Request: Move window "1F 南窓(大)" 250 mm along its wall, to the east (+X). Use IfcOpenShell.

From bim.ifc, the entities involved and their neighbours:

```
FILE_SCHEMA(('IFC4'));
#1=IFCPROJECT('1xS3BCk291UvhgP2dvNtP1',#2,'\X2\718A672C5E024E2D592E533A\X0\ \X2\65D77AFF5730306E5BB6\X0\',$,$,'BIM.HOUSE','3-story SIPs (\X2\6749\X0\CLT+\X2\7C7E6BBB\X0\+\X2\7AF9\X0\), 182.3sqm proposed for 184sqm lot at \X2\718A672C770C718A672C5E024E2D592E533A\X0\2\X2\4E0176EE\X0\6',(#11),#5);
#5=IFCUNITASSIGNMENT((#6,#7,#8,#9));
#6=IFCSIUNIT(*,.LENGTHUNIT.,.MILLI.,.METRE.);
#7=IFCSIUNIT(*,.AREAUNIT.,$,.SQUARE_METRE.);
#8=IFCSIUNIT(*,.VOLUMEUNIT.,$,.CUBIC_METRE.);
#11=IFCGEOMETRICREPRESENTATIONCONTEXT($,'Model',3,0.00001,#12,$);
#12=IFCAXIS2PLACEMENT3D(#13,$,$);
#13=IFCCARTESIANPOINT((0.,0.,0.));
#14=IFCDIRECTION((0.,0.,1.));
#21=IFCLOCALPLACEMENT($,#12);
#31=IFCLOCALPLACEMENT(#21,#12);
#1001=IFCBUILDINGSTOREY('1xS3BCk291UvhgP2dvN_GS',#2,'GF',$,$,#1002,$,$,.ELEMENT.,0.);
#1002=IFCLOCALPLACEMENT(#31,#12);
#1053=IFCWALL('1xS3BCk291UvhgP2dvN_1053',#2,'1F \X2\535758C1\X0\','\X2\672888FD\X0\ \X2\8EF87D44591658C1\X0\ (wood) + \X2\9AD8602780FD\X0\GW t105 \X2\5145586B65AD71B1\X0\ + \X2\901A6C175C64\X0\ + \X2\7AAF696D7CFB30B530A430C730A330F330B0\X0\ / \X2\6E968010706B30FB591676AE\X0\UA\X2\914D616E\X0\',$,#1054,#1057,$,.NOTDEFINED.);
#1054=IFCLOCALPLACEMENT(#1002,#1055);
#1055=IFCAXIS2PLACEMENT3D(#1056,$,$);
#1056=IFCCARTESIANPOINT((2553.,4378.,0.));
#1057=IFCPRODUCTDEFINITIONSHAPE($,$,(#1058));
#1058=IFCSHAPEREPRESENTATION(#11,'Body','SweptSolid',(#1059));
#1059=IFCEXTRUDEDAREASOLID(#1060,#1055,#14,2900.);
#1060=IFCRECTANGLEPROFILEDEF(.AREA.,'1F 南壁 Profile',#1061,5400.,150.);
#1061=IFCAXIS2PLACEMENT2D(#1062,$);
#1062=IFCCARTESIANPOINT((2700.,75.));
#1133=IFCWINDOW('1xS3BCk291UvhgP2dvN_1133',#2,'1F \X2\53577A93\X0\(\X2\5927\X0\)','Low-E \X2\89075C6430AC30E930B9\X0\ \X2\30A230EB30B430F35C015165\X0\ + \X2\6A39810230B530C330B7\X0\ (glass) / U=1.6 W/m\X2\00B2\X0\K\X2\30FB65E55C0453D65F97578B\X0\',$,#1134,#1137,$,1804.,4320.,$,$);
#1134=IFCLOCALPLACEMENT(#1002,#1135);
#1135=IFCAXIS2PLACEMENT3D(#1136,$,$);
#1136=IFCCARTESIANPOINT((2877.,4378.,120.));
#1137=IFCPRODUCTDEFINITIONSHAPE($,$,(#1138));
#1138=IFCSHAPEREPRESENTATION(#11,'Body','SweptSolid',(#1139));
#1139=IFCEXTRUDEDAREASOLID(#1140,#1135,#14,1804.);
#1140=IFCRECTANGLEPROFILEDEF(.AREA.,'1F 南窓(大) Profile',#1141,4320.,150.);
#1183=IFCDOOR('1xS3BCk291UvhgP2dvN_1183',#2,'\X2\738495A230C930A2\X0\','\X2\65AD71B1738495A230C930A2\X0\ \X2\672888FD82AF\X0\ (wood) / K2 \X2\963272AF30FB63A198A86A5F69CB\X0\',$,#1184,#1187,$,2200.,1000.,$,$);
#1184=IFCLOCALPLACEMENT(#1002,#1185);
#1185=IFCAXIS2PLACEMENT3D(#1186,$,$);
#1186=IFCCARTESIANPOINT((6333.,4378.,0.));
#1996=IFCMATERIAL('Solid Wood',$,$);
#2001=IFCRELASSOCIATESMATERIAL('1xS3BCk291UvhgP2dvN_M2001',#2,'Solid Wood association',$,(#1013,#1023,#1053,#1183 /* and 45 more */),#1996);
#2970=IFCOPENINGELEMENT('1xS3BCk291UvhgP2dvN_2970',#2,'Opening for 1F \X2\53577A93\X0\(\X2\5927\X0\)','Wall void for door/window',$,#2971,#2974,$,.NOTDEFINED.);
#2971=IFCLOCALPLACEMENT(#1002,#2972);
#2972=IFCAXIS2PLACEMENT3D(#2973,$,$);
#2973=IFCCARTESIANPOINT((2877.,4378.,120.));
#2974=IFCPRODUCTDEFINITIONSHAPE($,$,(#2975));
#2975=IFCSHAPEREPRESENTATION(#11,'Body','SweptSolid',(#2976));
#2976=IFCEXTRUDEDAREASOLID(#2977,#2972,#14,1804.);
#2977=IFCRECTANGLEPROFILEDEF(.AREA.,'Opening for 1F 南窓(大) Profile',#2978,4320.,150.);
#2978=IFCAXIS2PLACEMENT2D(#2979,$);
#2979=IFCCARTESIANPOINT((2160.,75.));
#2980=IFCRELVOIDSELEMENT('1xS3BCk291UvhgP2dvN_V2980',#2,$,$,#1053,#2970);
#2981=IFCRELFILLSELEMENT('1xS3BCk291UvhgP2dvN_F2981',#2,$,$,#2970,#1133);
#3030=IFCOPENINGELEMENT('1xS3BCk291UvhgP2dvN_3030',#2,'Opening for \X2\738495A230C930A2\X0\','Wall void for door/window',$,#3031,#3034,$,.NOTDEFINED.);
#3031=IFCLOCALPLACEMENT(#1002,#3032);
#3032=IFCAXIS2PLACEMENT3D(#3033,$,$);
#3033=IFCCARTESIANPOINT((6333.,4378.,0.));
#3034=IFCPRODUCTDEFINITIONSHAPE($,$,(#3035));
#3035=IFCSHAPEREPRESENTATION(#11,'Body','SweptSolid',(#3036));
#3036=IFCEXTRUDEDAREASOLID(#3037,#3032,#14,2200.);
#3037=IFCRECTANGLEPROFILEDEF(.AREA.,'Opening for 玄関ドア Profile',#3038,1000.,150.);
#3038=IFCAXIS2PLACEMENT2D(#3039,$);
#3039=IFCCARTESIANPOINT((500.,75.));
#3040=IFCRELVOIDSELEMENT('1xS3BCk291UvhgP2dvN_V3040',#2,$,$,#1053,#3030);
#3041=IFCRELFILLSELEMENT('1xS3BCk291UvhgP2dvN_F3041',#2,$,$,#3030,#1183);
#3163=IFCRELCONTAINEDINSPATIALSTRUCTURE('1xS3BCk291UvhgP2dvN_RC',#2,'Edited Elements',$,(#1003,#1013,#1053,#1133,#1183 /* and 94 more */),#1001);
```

```python
import ifcopenshell
import ifcopenshell.api.geometry
import ifcopenshell.util.placement
import ifcopenshell.util.unit

model = ifcopenshell.open("bim.ifc")
unit_scale = ifcopenshell.util.unit.calculate_unit_scale(model)

window = model.by_guid("1xS3BCk291UvhgP2dvN_1133")
opening = window.FillsVoids[0].RelatingOpeningElement
wall = opening.VoidsElements[0].RelatingBuildingElement

wall_matrix = ifcopenshell.util.placement.get_local_placement(wall.ObjectPlacement)
shift = wall_matrix[:3, 0] * 0.25 / unit_scale
before = ifcopenshell.util.placement.get_local_placement(window.ObjectPlacement)[:3, 3].copy()

# The window is not placed relative to its opening, so move both.
for product in (opening, window):
    matrix = ifcopenshell.util.placement.get_local_placement(product.ObjectPlacement)
    matrix[:3, 3] += shift
    ifcopenshell.api.geometry.edit_object_placement(model, product=product, matrix=matrix, is_si=False)

after = ifcopenshell.util.placement.get_local_placement(window.ObjectPlacement)[:3, 3]
print("window moved by", (after - before).round(3) + 0.0)

model.write("bim_edited.ifc")
```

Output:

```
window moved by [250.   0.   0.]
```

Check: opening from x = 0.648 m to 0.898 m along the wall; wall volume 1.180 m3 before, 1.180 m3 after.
